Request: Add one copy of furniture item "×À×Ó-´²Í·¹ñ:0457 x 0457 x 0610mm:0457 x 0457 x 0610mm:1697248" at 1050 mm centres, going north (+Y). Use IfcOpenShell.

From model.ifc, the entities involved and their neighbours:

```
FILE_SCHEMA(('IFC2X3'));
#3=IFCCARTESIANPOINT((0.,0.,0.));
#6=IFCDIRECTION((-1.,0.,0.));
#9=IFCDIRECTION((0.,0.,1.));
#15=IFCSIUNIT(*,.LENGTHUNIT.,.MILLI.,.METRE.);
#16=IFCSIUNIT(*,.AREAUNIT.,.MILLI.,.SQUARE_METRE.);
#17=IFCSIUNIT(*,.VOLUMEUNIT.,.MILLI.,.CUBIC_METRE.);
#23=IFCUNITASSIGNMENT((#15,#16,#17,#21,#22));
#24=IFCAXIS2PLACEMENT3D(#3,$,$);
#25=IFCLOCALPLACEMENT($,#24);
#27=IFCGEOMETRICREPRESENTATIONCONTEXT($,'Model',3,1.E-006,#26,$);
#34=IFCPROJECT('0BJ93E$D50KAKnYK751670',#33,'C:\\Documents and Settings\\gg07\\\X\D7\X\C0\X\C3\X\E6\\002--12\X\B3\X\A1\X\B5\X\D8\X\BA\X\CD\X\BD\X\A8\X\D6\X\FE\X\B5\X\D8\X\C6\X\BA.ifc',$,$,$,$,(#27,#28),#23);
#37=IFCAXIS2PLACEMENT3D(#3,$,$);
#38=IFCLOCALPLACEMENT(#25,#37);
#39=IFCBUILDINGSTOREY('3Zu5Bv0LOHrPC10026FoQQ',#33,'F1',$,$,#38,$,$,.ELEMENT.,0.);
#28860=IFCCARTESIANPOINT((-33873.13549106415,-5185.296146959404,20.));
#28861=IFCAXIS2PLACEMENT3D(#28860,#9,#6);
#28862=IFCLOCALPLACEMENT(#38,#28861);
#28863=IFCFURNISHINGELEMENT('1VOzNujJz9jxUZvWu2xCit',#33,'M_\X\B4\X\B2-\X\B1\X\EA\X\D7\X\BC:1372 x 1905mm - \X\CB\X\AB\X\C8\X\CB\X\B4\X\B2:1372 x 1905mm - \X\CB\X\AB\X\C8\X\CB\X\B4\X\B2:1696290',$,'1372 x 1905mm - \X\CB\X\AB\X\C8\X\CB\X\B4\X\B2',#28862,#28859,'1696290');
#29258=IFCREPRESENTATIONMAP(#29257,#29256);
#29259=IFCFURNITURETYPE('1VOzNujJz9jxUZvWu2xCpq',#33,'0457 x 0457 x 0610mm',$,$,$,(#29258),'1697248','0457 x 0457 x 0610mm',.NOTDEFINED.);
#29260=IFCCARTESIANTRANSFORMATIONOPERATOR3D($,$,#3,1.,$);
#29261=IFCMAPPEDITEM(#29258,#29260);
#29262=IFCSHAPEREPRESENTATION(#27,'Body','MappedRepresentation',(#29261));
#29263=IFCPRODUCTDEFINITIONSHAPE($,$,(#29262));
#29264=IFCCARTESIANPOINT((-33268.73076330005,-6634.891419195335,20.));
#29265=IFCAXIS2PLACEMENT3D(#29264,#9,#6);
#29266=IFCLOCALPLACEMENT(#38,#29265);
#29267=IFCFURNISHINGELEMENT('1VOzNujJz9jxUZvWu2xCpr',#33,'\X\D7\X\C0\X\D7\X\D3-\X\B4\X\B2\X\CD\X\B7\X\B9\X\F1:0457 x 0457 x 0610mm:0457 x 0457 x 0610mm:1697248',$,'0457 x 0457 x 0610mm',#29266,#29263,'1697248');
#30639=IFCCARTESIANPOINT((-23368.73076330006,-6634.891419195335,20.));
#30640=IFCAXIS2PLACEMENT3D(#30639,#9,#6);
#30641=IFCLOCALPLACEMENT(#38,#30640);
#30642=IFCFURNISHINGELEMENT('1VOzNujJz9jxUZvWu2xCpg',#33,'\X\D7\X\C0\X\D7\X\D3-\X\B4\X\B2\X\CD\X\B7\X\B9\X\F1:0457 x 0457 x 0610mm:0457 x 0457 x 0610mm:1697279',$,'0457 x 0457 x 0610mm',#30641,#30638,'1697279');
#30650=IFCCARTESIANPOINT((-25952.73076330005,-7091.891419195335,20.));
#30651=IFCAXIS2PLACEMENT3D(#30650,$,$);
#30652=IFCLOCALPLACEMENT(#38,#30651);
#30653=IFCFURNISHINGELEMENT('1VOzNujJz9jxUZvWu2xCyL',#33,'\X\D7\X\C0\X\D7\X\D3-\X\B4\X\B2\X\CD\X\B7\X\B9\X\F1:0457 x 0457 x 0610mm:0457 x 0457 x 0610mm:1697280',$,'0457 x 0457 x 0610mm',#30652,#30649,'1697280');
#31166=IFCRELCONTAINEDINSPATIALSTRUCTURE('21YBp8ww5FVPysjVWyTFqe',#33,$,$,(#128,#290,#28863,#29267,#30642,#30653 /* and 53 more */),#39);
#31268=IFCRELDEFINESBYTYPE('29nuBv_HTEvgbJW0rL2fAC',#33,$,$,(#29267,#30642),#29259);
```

```python
import numpy as np
import ifcopenshell
import ifcopenshell.api.geometry
import ifcopenshell.api.root
import ifcopenshell.util.element
import ifcopenshell.util.placement
import ifcopenshell.util.unit

model = ifcopenshell.open("model.ifc")
unit_scale = ifcopenshell.util.unit.calculate_unit_scale(model)


def reuse_history(source, copy):
    """copy_class also copies each property set's owner history, people and application; keep the originals."""
    for rel in copy.IsDefinedBy:
        if rel.is_a("IfcRelDefinesByProperties") and (history := rel.RelatingPropertyDefinition.OwnerHistory):
            rel.RelatingPropertyDefinition.OwnerHistory = source.OwnerHistory
            ifcopenshell.util.element.remove_deep2(model, history)


source = model.by_id(29267)
base = ifcopenshell.util.placement.get_local_placement(source.ObjectPlacement)
step = np.array([0.0, 1.0, 0.0]) * 1.05 / unit_scale

for i in range(1, 2):
    copy = ifcopenshell.api.root.copy_class(model, product=source)
    copy.Representation = ifcopenshell.util.element.copy_deep(
        model, source.Representation, exclude=["IfcGeometricRepresentationContext", "IfcRepresentationMap"]
    )
    copy.Name = "×À×Ó-´²Í·¹ñ:0457 x 0457 x 0610mm:0457 x 0457 x 0610mm"
    copy.Tag = None
    reuse_history(source, copy)
    matrix = base.copy()
    matrix[:3, 3] += i * step
    print("added at", matrix[:3, 3].round(3) + 0.0)
    ifcopenshell.api.geometry.edit_object_placement(model, product=copy, matrix=matrix, is_si=False)

model.write("model_rev.ifc")
```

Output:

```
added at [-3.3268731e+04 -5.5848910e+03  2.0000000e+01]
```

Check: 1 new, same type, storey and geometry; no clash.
